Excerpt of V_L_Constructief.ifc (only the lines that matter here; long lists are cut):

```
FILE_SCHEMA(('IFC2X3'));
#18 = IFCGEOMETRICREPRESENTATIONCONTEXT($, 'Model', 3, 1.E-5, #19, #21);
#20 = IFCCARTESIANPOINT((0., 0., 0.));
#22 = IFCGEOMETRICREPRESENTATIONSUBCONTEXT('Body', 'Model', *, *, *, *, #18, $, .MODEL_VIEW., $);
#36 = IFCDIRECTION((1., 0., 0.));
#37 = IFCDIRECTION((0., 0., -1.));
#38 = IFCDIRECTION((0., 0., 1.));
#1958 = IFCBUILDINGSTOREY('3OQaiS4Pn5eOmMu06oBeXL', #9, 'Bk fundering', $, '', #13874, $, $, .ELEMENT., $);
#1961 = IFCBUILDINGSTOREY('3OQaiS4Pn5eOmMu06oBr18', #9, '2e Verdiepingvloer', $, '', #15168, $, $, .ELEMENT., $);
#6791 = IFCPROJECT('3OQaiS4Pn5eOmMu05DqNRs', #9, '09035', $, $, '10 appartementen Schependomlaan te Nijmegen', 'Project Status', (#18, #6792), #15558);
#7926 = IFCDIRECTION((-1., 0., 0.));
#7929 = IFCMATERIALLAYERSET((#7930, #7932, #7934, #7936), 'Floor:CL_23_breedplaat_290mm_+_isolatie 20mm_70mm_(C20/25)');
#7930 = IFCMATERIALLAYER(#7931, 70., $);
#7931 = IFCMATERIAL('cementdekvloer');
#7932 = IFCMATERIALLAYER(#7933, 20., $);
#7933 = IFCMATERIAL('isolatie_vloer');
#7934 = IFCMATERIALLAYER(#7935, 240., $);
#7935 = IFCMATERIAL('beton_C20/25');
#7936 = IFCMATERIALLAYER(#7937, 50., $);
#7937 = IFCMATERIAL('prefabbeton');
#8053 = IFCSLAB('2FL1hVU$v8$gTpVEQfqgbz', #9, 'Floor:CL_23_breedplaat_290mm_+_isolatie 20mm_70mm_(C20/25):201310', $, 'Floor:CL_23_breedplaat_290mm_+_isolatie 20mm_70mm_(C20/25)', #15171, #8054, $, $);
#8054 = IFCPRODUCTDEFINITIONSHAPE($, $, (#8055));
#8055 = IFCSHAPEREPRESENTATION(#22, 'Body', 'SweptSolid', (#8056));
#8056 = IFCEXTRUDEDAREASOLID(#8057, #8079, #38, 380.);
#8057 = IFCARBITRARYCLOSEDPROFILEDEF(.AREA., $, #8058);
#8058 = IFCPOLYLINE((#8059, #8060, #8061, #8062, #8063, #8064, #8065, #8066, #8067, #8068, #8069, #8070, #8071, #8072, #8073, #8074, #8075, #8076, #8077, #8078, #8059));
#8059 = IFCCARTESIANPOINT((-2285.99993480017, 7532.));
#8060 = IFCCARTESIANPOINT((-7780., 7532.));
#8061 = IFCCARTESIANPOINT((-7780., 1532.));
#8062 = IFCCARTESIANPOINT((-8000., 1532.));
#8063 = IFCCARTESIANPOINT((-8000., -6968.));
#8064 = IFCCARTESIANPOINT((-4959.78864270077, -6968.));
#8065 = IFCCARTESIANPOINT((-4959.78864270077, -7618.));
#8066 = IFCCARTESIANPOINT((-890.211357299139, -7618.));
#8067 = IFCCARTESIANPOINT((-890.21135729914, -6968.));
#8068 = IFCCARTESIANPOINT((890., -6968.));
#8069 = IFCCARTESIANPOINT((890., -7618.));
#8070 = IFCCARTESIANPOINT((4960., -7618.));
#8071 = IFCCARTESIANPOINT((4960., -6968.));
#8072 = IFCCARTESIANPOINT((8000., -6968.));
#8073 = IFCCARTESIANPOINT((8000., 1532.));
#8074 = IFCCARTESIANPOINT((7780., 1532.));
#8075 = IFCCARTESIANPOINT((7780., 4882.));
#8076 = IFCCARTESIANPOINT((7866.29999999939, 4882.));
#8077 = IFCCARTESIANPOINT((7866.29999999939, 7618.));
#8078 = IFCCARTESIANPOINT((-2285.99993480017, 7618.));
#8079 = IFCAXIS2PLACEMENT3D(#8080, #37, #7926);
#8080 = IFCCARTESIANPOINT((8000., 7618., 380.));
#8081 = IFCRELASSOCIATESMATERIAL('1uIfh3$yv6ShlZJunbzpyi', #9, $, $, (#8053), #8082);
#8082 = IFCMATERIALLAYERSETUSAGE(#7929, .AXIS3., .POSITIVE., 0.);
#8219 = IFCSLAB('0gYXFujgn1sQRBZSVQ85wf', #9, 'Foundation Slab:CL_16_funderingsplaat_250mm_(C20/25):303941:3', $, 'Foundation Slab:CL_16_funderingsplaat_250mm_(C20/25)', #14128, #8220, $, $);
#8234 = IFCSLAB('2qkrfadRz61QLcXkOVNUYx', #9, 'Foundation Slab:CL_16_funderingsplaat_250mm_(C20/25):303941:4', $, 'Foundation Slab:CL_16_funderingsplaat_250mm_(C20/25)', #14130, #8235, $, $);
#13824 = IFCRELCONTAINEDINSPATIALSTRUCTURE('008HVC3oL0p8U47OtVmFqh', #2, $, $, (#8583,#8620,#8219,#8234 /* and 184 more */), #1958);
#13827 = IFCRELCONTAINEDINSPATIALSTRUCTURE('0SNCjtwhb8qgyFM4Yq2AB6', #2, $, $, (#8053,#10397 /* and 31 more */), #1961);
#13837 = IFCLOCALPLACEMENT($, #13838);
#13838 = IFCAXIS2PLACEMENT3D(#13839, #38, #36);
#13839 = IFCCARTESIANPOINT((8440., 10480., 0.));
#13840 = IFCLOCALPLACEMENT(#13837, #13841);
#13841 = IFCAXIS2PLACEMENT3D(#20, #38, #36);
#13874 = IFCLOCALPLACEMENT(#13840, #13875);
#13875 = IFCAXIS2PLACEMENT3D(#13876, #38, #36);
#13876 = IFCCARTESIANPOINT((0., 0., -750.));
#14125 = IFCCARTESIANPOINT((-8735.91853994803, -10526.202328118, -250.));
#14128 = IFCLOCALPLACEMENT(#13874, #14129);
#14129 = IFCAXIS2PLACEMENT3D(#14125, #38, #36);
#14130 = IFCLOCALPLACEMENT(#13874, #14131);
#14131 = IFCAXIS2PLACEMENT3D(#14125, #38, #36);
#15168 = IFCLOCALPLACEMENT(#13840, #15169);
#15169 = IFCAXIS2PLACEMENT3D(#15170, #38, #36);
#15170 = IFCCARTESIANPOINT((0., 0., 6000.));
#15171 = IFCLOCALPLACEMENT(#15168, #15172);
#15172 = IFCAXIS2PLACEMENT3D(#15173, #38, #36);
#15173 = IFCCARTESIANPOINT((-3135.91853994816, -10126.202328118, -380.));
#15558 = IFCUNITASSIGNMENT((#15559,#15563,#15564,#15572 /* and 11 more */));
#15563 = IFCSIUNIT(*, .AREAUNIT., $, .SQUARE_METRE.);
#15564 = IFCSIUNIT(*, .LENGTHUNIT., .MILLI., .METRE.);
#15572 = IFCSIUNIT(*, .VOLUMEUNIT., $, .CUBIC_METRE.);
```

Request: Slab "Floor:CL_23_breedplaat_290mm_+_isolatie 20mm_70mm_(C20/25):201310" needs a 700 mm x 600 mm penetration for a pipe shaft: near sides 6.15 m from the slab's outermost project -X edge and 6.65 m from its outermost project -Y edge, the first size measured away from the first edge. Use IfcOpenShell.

```python
import numpy as np
import ifcopenshell
import ifcopenshell.api.feature
import ifcopenshell.api.geometry
import ifcopenshell.api.root
import ifcopenshell.geom
import ifcopenshell.util.placement
import ifcopenshell.util.representation
import ifcopenshell.util.shape
import ifcopenshell.util.unit

model = ifcopenshell.open("V_L_Constructief.ifc")
unit_scale = ifcopenshell.util.unit.calculate_unit_scale(model)
settings = ifcopenshell.geom.settings()


def volume(element):
    """Net volume in cubic metres, openings subtracted."""
    shape = ifcopenshell.geom.create_shape(settings, element)
    return ifcopenshell.util.shape.get_volume(shape.geometry)


slab = model.by_id(8053)
before = volume(slab)

# Extent in the slab's own axes, in metres. The edges named are its -X and -Y sides.
slab_shape = ifcopenshell.geom.create_shape(settings, slab)
vertices = ifcopenshell.util.shape.get_vertices(slab_shape.geometry)
x_min, y_min, bottom = vertices.min(axis=0)
top = vertices[:, 2].max()

opening = ifcopenshell.api.root.create_entity(model, ifc_class="IfcOpeningElement", name="Pipe shaft opening")
context = ifcopenshell.util.representation.get_context(model, "Model", "Body", "MODEL_VIEW")
width, depth = 0.7, 0.6
outline = [(0.0, 0.0), (width, 0.0), (width, depth), (0.0, depth), (0.0, 0.0)]
# Overshoot both faces by 50 mm so the cut is clean.
shape = ifcopenshell.api.geometry.add_slab_representation(
    model, context=context, depth=top - bottom + 0.1, polyline=outline
)
ifcopenshell.api.geometry.assign_representation(model, product=opening, representation=shape)

matrix = ifcopenshell.util.placement.get_local_placement(slab.ObjectPlacement)
matrix[:, 3] = matrix @ np.append(np.array([x_min + 6.15, y_min + 6.65, bottom - 0.05]) / unit_scale, 1.0)
ifcopenshell.api.geometry.edit_object_placement(model, product=opening, matrix=matrix, is_si=False)
ifcopenshell.api.feature.add_feature(model, feature=opening, element=slab)

after = volume(slab)

print(f"slab volume {before:.3f} -> {after:.3f} m3")

model.write("V_L_Constructief-out.ifc")
```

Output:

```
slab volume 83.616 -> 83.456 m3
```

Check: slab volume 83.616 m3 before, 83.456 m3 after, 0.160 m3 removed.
